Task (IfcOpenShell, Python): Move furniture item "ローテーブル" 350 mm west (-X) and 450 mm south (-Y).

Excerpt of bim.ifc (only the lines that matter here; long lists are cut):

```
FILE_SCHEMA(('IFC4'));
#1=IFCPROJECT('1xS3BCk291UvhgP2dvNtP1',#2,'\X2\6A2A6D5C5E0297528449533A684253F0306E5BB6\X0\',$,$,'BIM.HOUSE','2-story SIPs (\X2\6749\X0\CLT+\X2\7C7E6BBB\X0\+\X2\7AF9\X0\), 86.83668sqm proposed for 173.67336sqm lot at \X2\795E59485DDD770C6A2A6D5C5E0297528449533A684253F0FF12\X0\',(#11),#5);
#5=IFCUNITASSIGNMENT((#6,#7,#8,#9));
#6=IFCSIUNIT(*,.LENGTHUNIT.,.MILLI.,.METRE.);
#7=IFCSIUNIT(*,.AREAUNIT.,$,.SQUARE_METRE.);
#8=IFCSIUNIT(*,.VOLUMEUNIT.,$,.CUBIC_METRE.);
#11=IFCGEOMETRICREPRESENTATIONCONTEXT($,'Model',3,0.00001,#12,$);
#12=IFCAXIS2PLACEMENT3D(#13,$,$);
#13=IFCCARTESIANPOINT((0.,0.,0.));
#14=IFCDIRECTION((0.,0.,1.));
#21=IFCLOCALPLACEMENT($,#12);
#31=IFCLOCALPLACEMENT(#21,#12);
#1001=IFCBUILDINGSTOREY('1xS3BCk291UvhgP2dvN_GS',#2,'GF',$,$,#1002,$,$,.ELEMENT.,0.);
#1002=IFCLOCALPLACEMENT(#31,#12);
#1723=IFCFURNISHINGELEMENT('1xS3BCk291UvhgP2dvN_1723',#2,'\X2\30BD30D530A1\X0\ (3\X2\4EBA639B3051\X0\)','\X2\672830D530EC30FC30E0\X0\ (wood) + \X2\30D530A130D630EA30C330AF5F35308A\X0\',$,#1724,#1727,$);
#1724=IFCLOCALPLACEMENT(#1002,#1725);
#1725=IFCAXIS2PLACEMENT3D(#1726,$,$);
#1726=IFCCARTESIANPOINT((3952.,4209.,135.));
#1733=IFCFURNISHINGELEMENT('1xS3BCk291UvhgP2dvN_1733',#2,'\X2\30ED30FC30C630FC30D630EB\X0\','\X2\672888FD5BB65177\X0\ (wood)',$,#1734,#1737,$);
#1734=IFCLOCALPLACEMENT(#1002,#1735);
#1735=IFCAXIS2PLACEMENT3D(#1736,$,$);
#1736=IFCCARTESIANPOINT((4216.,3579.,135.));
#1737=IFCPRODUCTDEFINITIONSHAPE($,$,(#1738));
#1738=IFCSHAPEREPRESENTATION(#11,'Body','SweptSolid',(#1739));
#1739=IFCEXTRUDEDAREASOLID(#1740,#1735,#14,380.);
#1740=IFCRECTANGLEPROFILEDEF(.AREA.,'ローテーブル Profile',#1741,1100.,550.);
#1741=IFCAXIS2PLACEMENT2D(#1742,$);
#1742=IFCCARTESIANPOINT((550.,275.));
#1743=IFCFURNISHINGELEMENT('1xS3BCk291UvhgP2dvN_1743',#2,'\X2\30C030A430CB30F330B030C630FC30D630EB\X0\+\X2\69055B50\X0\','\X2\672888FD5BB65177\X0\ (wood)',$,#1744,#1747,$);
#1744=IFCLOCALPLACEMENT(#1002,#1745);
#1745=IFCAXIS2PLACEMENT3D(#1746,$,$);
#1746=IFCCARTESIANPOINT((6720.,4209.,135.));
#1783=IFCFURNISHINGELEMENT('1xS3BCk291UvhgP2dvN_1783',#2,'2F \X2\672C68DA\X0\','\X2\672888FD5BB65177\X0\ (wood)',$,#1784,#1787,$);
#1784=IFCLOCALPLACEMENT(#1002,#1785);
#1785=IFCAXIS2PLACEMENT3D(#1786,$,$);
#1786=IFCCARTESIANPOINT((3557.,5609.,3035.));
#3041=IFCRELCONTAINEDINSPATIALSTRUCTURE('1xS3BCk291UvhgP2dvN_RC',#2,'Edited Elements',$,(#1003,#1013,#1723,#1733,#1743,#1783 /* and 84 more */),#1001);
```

```python
import ifcopenshell
import ifcopenshell.api.geometry
import ifcopenshell.util.placement

model = ifcopenshell.open("bim.ifc")

item = model.by_guid("1xS3BCk291UvhgP2dvN_1733")
matrix = ifcopenshell.util.placement.get_local_placement(item.ObjectPlacement)
matrix[0, 3] -= 350.0
matrix[1, 3] -= 450.0
ifcopenshell.api.geometry.edit_object_placement(model, product=item, matrix=matrix, is_si=False)

print(ifcopenshell.util.placement.get_local_placement(item.ObjectPlacement).round(3) + 0.0)

model.write("bim-out.ifc")
```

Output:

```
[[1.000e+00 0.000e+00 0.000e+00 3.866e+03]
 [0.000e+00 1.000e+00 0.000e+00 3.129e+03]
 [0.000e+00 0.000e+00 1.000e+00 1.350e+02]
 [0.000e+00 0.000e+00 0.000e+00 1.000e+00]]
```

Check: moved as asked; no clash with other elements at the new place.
